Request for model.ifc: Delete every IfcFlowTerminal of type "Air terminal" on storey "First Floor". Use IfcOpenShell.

First a look at what the model holds.

```python
import ifcopenshell
import ifcopenshell.util.element

model = ifcopenshell.open("model.ifc")
print(model.schema)
storey = next(s for s in model.by_type("IfcBuildingStorey") if s.Name == "First Floor")
terminals = [e for e in ifcopenshell.util.element.get_decomposition(storey) if e.is_a("IfcFlowTerminal")]
seen = {}
for e in terminals:
    element_type = ifcopenshell.util.element.get_type(e)
    name = element_type.Name if element_type not in (None, e) else None
    seen[name] = seen.get(name, 0) + 1
for name, count in sorted(seen.items(), key=str):
    print(count, "x", name)
```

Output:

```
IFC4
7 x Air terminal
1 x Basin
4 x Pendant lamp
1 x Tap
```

```python
import ifcopenshell
import ifcopenshell.api.root
import ifcopenshell.util.element

model = ifcopenshell.open("model.ifc")

storey = next(s for s in model.by_type("IfcBuildingStorey") if s.Name == "First Floor")
terminals = [e for e in ifcopenshell.util.element.get_decomposition(storey) if e.is_a("IfcFlowTerminal")]
targets = [e for e in terminals if (t := ifcopenshell.util.element.get_type(e)) not in (None, e) and t.Name == "Air terminal"]

for e in targets:
    ifcopenshell.api.root.remove_product(model, product=e)
print(len(targets), "removed")

model.write("model_v2.ifc")
```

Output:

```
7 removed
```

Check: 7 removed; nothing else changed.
